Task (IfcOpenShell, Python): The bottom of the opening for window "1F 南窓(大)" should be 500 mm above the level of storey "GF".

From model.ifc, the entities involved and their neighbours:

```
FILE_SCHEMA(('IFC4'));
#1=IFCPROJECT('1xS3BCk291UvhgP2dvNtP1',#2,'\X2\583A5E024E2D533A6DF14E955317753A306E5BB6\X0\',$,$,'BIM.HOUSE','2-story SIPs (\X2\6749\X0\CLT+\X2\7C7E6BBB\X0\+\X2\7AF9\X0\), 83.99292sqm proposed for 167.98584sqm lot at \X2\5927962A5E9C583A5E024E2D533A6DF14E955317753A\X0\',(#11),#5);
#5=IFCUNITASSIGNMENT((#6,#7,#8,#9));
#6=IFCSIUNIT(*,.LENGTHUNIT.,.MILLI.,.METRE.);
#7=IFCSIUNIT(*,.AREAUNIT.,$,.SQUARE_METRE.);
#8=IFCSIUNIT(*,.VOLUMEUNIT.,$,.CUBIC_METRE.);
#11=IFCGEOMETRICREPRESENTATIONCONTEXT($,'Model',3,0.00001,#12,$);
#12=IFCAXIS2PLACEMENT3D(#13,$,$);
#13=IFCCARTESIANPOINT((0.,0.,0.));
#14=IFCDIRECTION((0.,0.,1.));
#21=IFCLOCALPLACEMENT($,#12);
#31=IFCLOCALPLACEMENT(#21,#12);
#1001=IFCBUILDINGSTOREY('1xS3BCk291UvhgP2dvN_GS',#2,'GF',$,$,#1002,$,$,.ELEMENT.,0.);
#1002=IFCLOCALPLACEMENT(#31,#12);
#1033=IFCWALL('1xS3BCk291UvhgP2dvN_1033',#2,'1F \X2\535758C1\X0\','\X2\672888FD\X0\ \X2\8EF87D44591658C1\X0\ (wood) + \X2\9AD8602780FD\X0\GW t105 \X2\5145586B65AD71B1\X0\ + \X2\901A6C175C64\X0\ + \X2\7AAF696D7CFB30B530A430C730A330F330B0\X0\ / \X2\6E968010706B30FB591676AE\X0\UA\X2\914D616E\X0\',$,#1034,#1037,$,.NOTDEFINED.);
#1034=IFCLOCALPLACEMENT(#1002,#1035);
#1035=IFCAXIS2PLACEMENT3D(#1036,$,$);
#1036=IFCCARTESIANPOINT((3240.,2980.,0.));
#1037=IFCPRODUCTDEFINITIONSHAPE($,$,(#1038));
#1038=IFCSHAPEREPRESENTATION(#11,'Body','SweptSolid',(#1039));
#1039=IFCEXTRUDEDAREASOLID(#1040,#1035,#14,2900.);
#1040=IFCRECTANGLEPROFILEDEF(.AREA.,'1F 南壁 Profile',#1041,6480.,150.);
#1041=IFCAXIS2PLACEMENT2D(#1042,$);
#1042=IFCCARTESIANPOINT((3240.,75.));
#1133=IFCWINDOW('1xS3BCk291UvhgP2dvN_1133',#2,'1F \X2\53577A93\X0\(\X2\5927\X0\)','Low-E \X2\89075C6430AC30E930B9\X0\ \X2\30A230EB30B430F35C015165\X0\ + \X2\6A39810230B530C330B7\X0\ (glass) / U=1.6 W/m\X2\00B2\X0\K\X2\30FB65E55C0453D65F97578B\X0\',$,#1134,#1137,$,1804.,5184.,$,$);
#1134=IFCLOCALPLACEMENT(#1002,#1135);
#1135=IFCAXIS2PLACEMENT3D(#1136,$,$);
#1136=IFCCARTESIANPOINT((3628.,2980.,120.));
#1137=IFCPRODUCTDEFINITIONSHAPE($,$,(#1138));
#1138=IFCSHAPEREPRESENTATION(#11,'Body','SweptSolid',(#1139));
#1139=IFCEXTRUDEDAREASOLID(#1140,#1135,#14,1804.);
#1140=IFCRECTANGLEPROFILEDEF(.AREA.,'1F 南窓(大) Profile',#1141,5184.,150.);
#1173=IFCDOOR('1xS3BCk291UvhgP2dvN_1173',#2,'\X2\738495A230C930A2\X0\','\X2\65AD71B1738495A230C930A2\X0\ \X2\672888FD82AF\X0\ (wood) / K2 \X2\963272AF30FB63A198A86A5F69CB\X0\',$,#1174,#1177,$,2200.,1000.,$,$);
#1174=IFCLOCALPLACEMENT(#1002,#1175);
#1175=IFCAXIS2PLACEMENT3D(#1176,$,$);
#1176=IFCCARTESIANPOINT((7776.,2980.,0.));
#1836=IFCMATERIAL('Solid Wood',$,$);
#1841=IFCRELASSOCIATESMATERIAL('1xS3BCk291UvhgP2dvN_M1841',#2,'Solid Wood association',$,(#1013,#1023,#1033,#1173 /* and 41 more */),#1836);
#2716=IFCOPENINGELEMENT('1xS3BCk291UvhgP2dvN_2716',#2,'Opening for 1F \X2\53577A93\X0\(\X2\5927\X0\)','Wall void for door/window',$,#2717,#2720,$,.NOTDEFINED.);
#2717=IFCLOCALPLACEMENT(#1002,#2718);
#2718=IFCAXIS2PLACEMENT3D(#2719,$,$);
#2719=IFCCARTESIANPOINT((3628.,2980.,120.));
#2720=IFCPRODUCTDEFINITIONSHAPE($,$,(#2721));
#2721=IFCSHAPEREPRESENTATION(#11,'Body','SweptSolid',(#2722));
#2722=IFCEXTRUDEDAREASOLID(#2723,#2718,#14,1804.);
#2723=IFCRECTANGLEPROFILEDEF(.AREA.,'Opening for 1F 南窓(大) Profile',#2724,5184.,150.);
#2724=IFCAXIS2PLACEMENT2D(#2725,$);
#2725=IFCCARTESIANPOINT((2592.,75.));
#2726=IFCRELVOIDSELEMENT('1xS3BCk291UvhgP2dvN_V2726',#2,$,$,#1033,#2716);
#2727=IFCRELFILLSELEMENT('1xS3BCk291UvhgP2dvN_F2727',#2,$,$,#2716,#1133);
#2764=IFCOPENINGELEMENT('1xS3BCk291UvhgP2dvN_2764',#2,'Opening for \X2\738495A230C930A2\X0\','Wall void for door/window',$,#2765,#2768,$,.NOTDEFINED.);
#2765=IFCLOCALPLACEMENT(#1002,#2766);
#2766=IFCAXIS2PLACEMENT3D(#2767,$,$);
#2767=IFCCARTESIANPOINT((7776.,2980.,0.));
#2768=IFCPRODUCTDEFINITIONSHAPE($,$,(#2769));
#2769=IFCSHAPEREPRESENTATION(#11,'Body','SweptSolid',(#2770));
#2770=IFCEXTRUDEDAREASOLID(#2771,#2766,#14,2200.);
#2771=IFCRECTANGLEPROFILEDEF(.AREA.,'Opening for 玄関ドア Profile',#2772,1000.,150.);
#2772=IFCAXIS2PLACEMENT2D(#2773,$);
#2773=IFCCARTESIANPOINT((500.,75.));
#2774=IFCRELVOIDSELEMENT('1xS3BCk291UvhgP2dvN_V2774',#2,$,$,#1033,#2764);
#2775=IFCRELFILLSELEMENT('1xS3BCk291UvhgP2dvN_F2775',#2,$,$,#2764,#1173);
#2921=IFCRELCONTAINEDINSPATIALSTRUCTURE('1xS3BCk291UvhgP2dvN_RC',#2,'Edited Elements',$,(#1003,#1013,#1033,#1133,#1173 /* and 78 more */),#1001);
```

```python
import numpy as np
import ifcopenshell
import ifcopenshell.api.geometry
import ifcopenshell.geom
import ifcopenshell.util.element
import ifcopenshell.util.placement
import ifcopenshell.util.shape
import ifcopenshell.util.unit

model = ifcopenshell.open("model.ifc")
unit_scale = ifcopenshell.util.unit.calculate_unit_scale(model)

window = model.by_id(1133)
opening = window.FillsVoids[0].RelatingOpeningElement
storey = ifcopenshell.util.element.get_container(window, ifc_class="IfcBuildingStorey")
level = ifcopenshell.util.placement.get_local_placement(storey.ObjectPlacement)[2, 3]

# The opening's origin need not be at the sill, so measure its lowest point.
shape = ifcopenshell.geom.create_shape(ifcopenshell.geom.settings(), opening)
bottom = ifcopenshell.util.shape.get_shape_bottom_elevation(shape, shape.geometry) / unit_scale
dz = level + 0.5 / unit_scale - bottom

shift = np.array([0.0, 0.0, dz])
# The window is not placed relative to its opening, so move both.
for product in (opening, window):
    matrix = ifcopenshell.util.placement.get_local_placement(product.ObjectPlacement)
    matrix[:3, 3] += shift
    ifcopenshell.api.geometry.edit_object_placement(model, product=product, matrix=matrix, is_si=False)

print(f"moved by {dz * unit_scale:+.3f} m")

model.write("model_updated.ifc")
```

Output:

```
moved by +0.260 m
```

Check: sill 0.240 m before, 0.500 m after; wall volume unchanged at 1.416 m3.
